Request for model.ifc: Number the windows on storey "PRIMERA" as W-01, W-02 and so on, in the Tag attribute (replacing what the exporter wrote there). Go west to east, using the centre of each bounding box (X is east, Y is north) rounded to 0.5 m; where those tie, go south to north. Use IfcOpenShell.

First a look at what the model holds.

```python
import ifcopenshell
import ifcopenshell.util.element
import ifcopenshell.util.placement

model = ifcopenshell.open("model.ifc")
print(model.schema)
storey = next(s for s in model.by_type("IfcBuildingStorey") if s.Name == "PRIMERA")
windows = [e for e in ifcopenshell.util.element.get_decomposition(storey) if e.is_a("IfcWindow")]
for e in sorted(windows, key=lambda e: e.id()):
    origin = ifcopenshell.util.placement.get_local_placement(e.ObjectPlacement)[:3, 3]
    print(e.id(), e.Tag, e.Name, origin.round(2) + 0.0, sep=" | ")
```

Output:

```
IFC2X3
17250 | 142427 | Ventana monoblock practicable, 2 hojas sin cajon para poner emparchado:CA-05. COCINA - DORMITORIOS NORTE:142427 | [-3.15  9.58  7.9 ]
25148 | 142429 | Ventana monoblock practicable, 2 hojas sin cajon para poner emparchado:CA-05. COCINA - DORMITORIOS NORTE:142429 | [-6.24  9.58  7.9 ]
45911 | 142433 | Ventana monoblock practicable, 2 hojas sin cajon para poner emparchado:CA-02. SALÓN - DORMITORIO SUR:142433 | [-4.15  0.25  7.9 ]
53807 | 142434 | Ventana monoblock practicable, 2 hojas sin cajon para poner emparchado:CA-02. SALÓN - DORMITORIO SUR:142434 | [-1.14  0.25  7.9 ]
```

```python
import ifcopenshell
import ifcopenshell.geom
import ifcopenshell.util.element
import ifcopenshell.util.shape

model = ifcopenshell.open("model.ifc")
settings = ifcopenshell.geom.settings()
settings.set("use-world-coords", True)


def centre(element):
    shape = ifcopenshell.geom.create_shape(settings, element)
    return ifcopenshell.util.shape.get_bbox_centroid(shape.geometry)


storey = next(s for s in model.by_type("IfcBuildingStorey") if s.Name == "PRIMERA")
windows = [e for e in ifcopenshell.util.element.get_decomposition(storey) if e.is_a("IfcWindow")]

# Insertion points can sit at a corner or the storey origin, so sort by the geometry (in metres).
centres = {e: centre(e) for e in windows}
windows.sort(key=lambda e: (round(centres[e][0] / 0.5), centres[e][1]))

for i, e in enumerate(windows, start=1):
    number = f"W-{i:02d}"
    e.Tag = number
    print(e.id(), number)

model.write("model_edited.ifc")
```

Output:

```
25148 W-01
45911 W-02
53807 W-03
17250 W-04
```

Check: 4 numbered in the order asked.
